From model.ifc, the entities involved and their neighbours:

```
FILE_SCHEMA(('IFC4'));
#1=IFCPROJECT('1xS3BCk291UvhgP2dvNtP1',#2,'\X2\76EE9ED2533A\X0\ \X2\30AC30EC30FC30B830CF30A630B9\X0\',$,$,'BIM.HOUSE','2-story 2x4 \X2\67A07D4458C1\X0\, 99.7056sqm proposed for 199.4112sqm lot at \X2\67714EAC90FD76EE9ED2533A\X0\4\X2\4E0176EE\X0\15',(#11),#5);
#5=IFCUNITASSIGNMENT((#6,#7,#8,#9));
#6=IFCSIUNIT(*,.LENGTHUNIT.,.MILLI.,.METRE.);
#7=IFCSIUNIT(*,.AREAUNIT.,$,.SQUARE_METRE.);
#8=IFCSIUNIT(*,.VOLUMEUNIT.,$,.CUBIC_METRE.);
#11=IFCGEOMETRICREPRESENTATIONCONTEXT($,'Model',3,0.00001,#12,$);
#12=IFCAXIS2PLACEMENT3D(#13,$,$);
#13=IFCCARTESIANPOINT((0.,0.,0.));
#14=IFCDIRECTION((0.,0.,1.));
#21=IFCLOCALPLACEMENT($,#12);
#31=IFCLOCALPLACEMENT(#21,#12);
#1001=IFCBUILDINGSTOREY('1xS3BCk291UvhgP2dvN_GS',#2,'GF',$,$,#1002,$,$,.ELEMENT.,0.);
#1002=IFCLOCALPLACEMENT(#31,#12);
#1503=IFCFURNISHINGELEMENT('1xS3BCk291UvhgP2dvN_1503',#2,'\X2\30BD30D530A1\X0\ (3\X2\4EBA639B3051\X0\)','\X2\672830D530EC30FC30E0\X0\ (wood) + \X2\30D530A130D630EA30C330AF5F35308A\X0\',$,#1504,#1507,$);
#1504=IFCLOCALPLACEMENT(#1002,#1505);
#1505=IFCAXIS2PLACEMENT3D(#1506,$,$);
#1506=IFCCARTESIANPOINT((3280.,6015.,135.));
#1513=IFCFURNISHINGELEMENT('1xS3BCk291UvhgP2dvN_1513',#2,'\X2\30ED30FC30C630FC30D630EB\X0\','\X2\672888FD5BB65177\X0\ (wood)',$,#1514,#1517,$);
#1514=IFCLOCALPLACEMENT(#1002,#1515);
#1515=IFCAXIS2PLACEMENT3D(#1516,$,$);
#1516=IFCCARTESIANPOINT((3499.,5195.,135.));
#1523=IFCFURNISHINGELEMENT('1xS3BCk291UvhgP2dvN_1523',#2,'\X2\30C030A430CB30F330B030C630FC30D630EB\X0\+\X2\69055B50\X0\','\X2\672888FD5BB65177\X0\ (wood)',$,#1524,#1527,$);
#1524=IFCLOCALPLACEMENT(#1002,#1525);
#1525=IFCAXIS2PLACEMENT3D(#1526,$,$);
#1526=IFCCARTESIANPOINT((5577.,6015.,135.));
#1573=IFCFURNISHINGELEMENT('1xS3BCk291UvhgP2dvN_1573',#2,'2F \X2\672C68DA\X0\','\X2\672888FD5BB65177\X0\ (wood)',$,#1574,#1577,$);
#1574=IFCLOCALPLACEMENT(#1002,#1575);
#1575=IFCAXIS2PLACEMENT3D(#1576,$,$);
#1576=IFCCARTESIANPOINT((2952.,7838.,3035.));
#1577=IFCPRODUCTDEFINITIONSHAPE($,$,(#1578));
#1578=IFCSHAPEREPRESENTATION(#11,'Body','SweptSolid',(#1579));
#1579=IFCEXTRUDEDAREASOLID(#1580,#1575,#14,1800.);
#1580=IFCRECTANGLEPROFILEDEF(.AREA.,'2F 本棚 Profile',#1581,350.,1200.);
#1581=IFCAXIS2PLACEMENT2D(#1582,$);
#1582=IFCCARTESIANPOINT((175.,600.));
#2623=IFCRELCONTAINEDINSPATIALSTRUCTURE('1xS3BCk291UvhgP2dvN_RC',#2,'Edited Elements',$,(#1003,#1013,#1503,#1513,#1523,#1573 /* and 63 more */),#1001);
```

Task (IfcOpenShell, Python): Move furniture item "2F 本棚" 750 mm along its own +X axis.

```python
import ifcopenshell
import ifcopenshell.api.geometry
import ifcopenshell.util.placement
import ifcopenshell.util.unit

model = ifcopenshell.open("model.ifc")
unit_scale = ifcopenshell.util.unit.calculate_unit_scale(model)

item = model.by_id(1573)
matrix = ifcopenshell.util.placement.get_local_placement(item.ObjectPlacement)
matrix[:3, 3] += matrix[:3, 0] * 0.75 / unit_scale
ifcopenshell.api.geometry.edit_object_placement(model, product=item, matrix=matrix, is_si=False)

print(ifcopenshell.util.placement.get_local_placement(item.ObjectPlacement).round(3) + 0.0)

model.write("model_updated.ifc")
```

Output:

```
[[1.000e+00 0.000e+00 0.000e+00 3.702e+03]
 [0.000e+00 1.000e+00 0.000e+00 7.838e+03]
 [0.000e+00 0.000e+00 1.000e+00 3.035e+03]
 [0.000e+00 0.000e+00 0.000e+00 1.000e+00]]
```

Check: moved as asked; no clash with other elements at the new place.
